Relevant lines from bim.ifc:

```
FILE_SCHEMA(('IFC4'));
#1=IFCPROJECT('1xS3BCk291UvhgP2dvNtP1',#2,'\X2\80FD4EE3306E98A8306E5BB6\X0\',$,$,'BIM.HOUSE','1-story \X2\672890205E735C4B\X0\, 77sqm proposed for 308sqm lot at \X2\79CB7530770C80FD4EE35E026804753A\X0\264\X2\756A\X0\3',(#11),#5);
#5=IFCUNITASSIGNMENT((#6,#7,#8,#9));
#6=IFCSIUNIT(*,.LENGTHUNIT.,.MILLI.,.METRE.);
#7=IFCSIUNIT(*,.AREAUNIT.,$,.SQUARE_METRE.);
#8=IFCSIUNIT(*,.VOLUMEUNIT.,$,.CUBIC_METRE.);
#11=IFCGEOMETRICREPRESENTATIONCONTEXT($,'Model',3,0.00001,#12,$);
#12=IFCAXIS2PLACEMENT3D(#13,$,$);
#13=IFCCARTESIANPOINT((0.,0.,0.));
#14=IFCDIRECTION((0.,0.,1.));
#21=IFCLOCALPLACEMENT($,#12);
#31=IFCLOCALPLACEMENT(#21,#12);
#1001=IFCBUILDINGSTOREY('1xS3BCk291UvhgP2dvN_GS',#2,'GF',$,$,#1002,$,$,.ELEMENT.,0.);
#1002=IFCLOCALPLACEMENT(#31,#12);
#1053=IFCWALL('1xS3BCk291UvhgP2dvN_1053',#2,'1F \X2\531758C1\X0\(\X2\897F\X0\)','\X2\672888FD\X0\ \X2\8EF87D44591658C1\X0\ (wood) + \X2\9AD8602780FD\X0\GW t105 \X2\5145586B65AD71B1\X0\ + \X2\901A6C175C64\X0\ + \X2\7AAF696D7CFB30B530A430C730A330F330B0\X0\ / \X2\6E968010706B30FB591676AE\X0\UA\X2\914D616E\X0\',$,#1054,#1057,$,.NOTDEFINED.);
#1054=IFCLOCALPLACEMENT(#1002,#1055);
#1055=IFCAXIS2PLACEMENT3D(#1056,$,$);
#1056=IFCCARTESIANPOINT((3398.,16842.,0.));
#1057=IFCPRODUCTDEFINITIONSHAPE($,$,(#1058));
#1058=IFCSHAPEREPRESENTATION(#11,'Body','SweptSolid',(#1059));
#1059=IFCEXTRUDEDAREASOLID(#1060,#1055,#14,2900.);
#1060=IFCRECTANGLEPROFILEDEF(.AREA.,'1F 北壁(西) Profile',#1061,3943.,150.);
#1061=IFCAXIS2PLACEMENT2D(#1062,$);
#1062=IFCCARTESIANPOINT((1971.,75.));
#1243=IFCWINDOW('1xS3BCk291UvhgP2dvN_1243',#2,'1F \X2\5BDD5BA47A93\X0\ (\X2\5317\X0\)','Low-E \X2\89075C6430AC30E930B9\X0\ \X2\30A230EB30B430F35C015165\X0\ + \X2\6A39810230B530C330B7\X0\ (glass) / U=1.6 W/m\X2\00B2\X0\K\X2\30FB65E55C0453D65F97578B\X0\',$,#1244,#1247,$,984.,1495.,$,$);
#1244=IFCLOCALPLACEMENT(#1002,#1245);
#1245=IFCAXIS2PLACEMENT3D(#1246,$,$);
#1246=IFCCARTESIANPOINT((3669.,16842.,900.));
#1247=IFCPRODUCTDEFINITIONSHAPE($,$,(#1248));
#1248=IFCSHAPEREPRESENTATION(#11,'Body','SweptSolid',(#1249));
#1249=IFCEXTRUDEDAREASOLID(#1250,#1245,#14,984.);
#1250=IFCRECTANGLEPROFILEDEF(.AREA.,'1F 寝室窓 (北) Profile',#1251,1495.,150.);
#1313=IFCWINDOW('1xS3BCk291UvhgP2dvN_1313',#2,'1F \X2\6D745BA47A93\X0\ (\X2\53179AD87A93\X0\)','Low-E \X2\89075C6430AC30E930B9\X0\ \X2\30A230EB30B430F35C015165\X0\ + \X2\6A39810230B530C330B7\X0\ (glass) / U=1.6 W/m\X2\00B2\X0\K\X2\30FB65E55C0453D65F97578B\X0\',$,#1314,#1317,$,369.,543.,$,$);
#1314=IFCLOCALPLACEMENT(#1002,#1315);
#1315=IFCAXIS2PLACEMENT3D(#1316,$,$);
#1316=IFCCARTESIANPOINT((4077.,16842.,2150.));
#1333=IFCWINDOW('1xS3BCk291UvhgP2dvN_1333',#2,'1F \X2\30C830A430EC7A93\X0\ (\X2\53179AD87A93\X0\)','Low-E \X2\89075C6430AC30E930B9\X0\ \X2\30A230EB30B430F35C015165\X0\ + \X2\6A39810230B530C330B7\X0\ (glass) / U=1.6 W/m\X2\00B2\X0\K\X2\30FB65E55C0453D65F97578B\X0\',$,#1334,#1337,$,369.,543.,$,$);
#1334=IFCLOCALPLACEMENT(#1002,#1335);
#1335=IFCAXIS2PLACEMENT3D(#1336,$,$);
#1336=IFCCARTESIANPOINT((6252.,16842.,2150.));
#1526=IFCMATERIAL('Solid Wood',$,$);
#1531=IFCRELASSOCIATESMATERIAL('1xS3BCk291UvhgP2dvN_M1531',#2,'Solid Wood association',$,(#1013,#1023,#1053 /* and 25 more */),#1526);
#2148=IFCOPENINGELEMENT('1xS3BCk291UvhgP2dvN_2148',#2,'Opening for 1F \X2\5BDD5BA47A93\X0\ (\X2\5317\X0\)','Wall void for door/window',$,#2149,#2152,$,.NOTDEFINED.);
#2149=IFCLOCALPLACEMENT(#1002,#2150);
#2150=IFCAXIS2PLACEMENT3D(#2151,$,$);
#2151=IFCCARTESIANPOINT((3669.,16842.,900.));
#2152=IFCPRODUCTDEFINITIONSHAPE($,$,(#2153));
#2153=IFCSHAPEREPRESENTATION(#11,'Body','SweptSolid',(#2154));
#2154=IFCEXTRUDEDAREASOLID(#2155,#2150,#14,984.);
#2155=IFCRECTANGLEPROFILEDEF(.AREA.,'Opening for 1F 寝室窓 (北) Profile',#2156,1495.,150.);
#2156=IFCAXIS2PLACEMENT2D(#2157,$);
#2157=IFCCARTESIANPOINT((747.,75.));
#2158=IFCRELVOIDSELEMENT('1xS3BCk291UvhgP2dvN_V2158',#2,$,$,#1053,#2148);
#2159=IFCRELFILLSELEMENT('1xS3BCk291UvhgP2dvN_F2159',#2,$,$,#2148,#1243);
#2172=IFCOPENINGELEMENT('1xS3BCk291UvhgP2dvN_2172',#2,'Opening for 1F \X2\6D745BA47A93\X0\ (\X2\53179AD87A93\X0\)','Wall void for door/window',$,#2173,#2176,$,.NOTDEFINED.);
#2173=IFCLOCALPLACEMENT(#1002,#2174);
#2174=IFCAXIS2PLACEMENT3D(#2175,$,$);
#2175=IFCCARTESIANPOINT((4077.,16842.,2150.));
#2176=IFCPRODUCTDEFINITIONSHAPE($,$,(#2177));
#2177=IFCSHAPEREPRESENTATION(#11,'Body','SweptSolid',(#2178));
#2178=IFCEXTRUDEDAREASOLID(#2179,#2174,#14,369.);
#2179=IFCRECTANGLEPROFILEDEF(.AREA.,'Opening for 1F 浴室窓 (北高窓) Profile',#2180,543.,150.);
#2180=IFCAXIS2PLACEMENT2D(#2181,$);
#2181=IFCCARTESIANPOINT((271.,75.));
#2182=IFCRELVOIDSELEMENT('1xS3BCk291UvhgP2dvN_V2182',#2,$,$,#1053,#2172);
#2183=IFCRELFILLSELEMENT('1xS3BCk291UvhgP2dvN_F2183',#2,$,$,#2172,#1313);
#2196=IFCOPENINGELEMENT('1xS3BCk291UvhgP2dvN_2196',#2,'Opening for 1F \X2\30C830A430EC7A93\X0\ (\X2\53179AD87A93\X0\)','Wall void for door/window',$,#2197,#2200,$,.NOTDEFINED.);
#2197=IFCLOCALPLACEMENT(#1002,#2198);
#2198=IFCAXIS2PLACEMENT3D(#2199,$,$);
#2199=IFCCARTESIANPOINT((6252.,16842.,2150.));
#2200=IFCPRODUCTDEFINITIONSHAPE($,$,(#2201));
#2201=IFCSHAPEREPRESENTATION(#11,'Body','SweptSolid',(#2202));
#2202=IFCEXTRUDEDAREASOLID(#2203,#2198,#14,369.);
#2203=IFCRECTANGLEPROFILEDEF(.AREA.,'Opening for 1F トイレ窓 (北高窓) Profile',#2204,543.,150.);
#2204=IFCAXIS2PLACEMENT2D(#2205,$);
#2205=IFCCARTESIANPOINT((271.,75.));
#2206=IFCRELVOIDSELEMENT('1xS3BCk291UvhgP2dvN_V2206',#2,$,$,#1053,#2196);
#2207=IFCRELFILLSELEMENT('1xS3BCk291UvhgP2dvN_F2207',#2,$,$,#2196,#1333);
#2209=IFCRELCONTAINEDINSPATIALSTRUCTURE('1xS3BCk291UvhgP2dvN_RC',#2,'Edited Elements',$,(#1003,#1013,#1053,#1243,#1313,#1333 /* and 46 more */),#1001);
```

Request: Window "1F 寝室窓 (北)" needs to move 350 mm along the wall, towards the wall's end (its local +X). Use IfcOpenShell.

```python
import ifcopenshell
import ifcopenshell.api.geometry
import ifcopenshell.util.placement
import ifcopenshell.util.unit

model = ifcopenshell.open("bim.ifc")
unit_scale = ifcopenshell.util.unit.calculate_unit_scale(model)

window = model.by_guid("1xS3BCk291UvhgP2dvN_1243")
opening = window.FillsVoids[0].RelatingOpeningElement
wall = opening.VoidsElements[0].RelatingBuildingElement

wall_matrix = ifcopenshell.util.placement.get_local_placement(wall.ObjectPlacement)
shift = wall_matrix[:3, 0] * 0.35 / unit_scale
before = ifcopenshell.util.placement.get_local_placement(window.ObjectPlacement)[:3, 3].copy()

# The window is not placed relative to its opening, so move both.
for product in (opening, window):
    matrix = ifcopenshell.util.placement.get_local_placement(product.ObjectPlacement)
    matrix[:3, 3] += shift
    ifcopenshell.api.geometry.edit_object_placement(model, product=product, matrix=matrix, is_si=False)

after = ifcopenshell.util.placement.get_local_placement(window.ObjectPlacement)[:3, 3]
print("window moved by", (after - before).round(3) + 0.0)

model.write("bim-out.ifc")
```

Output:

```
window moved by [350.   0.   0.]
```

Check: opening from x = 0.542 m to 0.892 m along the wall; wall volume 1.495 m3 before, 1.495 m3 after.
